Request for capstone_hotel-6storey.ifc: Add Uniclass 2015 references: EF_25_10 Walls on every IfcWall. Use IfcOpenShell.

First a look at what the model holds.

```python
import ifcopenshell

model = ifcopenshell.open("capstone_hotel-6storey.ifc")
print(model.schema)
print("classifications:", [c.Name for c in model.by_type("IfcClassification")])
for ifc_class in ("IfcDoor", "IfcRoof", "IfcStair", "IfcWall", "IfcWindow"):
    print(ifc_class, len(model.by_type(ifc_class)))
```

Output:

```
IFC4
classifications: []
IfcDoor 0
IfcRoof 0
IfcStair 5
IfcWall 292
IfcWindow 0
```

```python
import ifcopenshell
import ifcopenshell.api.classification

model = ifcopenshell.open("capstone_hotel-6storey.ifc")

system = ifcopenshell.api.classification.add_classification(model, classification="Uniclass 2015")

codes = {
    "IfcWall": ("EF_25_10", "Walls"),
}
for ifc_class, (code, name) in codes.items():
    products = model.by_type(ifc_class)
    ifcopenshell.api.classification.add_reference(
        model, products=products, classification=system, identification=code, name=name
    )
    print(code, len(products))

model.write("capstone_hotel-6storey_edited.ifc")
```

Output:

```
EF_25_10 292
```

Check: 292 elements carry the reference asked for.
